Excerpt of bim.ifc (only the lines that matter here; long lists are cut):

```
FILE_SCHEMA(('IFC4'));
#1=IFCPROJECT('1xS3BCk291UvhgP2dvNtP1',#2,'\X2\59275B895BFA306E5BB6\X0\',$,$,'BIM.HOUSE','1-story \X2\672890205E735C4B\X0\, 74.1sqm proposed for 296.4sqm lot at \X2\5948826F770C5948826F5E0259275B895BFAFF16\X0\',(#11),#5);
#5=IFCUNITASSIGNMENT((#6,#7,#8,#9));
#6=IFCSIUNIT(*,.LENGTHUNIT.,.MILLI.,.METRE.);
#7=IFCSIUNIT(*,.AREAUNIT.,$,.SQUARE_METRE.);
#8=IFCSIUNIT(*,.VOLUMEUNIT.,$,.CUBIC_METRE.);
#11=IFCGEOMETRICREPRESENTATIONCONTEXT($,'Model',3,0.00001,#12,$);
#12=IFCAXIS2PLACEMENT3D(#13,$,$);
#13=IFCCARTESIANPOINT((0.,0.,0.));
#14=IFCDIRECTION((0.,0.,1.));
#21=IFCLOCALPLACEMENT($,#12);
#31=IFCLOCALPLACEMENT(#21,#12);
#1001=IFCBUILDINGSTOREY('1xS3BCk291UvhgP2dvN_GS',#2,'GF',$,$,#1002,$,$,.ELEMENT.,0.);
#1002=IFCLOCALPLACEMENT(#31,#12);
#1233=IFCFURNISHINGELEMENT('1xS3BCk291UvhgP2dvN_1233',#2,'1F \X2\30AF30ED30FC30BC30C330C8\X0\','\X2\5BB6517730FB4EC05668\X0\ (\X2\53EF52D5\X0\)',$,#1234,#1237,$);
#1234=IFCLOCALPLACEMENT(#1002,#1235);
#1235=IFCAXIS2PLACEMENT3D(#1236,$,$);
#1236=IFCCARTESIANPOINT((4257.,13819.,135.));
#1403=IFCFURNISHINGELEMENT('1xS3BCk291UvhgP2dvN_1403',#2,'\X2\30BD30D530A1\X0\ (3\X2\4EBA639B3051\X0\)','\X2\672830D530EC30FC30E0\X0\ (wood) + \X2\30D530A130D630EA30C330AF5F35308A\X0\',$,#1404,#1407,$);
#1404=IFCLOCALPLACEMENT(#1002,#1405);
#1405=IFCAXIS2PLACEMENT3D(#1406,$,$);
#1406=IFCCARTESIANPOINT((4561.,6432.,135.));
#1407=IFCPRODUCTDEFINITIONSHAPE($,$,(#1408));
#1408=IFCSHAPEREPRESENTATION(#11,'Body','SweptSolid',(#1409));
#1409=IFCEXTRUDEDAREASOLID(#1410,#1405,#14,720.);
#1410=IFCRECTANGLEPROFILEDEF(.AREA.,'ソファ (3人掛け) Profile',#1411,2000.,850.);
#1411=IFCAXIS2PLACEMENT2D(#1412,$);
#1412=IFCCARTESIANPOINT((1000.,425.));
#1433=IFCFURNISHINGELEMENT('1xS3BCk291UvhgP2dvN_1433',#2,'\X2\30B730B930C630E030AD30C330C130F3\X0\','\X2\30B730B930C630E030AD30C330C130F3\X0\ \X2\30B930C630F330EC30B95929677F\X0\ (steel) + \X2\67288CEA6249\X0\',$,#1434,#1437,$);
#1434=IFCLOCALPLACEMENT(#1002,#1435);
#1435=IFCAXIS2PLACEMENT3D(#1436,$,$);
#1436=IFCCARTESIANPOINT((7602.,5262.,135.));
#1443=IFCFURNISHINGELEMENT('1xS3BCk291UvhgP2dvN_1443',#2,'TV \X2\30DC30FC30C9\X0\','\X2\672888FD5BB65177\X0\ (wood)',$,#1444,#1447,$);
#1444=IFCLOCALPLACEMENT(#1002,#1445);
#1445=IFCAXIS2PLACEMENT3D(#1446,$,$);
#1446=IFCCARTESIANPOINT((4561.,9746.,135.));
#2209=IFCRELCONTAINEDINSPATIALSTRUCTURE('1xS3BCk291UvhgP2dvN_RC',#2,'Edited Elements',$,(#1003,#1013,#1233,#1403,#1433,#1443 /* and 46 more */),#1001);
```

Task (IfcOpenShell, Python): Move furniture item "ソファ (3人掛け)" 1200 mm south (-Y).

```python
import ifcopenshell
import ifcopenshell.api.geometry
import ifcopenshell.util.placement
import ifcopenshell.util.unit

model = ifcopenshell.open("bim.ifc")
unit_scale = ifcopenshell.util.unit.calculate_unit_scale(model)

item = model.by_guid("1xS3BCk291UvhgP2dvN_1403")
matrix = ifcopenshell.util.placement.get_local_placement(item.ObjectPlacement)
matrix[1, 3] -= 1.2 / unit_scale
ifcopenshell.api.geometry.edit_object_placement(model, product=item, matrix=matrix, is_si=False)

print(ifcopenshell.util.placement.get_local_placement(item.ObjectPlacement).round(3) + 0.0)

model.write("bim_rev.ifc")
```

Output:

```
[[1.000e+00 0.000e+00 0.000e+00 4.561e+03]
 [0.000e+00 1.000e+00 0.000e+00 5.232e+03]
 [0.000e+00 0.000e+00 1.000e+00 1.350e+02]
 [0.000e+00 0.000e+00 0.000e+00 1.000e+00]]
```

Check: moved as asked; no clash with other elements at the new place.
